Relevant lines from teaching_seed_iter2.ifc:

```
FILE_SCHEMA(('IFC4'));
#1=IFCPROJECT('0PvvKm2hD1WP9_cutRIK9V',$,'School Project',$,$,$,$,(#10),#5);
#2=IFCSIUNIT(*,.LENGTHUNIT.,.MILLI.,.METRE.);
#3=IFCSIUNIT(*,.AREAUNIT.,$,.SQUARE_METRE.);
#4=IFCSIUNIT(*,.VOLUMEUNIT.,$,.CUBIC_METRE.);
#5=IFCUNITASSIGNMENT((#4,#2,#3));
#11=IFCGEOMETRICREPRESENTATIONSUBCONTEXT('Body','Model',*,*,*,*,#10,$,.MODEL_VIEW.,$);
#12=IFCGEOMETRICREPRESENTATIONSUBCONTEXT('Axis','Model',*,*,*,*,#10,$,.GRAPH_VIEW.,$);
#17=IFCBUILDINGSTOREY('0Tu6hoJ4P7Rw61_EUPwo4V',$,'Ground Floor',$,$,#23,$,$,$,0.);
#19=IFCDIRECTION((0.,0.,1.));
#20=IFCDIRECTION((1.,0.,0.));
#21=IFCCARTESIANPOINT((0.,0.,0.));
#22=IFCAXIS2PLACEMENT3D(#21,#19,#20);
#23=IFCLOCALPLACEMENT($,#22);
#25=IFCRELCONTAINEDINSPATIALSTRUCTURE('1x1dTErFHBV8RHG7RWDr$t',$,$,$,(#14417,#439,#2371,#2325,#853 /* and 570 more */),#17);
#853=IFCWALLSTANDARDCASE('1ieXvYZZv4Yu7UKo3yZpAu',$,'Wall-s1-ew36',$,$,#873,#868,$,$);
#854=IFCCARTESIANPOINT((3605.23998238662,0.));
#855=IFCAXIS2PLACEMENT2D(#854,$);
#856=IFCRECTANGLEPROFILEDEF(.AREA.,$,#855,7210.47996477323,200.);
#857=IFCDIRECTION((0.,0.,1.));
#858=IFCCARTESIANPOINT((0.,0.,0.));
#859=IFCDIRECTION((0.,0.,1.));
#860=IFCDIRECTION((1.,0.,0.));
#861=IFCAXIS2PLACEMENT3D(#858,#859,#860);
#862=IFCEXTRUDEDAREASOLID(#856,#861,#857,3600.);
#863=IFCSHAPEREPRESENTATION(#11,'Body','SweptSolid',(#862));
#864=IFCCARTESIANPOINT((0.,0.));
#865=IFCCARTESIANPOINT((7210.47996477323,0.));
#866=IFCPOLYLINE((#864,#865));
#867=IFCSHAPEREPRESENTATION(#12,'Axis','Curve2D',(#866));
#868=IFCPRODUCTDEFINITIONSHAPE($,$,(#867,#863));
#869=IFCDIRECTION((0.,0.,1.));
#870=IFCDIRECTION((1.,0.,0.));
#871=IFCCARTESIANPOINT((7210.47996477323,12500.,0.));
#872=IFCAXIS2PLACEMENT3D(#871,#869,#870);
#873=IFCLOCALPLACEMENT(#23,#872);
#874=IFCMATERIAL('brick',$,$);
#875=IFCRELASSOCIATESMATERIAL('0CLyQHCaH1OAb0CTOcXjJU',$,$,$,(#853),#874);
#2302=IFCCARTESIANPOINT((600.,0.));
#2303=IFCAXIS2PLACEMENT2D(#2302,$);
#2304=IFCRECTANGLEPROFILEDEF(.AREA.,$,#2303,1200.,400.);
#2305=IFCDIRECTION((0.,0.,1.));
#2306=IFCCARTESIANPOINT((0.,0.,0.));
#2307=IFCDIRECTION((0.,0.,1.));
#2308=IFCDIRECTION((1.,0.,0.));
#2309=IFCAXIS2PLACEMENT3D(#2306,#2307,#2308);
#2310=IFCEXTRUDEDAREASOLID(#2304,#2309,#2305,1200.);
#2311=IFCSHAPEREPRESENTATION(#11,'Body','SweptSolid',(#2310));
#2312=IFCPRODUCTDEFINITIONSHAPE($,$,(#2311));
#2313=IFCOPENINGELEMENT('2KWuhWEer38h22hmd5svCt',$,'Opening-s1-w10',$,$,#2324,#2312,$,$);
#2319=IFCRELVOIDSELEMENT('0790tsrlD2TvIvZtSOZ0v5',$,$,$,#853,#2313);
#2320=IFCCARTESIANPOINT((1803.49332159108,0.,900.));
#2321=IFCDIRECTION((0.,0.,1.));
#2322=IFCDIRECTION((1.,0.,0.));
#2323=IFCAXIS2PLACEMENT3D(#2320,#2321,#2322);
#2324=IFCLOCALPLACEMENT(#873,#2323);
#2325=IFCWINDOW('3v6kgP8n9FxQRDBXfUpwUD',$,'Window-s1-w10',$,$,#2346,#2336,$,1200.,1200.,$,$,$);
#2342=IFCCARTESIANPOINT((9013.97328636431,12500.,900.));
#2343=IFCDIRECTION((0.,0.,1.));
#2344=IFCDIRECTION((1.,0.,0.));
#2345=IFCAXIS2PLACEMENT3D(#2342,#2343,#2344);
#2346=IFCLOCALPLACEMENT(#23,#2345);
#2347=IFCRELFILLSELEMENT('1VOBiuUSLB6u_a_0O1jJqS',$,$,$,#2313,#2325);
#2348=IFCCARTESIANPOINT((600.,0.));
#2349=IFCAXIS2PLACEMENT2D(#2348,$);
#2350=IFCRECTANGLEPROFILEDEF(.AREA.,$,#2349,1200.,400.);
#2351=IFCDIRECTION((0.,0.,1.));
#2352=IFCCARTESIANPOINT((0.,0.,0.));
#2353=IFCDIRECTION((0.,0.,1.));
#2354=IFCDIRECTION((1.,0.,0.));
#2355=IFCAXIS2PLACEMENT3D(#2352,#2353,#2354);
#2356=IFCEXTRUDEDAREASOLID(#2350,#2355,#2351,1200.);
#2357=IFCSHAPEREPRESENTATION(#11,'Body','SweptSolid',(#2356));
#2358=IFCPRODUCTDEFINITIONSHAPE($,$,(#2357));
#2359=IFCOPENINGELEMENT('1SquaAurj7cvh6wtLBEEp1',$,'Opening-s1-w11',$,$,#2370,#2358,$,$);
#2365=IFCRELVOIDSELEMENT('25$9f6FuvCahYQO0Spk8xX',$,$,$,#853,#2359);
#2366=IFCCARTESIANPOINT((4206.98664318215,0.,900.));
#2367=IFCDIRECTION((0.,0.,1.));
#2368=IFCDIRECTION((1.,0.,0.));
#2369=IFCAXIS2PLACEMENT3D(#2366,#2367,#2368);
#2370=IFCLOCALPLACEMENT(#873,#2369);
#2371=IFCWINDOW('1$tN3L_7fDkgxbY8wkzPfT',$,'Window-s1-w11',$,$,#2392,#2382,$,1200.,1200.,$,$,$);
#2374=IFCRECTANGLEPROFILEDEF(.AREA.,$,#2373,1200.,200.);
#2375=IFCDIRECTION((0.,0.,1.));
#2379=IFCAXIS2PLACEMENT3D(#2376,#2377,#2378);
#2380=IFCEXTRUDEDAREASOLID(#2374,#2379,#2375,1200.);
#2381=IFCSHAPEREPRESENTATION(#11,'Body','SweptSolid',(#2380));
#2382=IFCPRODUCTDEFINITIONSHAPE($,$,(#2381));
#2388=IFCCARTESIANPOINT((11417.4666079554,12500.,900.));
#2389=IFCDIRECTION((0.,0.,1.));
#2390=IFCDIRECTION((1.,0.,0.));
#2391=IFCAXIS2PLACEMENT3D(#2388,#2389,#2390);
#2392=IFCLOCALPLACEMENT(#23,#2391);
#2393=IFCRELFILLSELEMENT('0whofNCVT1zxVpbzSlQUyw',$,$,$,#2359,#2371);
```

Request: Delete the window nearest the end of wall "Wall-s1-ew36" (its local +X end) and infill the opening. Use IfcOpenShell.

```python
import ifcopenshell
import ifcopenshell.api.feature
import ifcopenshell.api.root
import ifcopenshell.geom
import ifcopenshell.util.shape

model = ifcopenshell.open("teaching_seed_iter2.ifc")
settings = ifcopenshell.geom.settings()


def volume(element):
    """Net volume in cubic metres, openings subtracted."""
    shape = ifcopenshell.geom.create_shape(settings, element)
    return ifcopenshell.util.shape.get_volume(shape.geometry)


window = model.by_guid("1$tN3L_7fDkgxbY8wkzPfT")
opening = window.FillsVoids[0].RelatingOpeningElement
wall = opening.VoidsElements[0].RelatingBuildingElement
before = volume(wall)

ifcopenshell.api.root.remove_product(model, product=window)
ifcopenshell.api.feature.remove_feature(model, feature=opening)

after = volume(wall)

print(f"wall volume {before:.3f} -> {after:.3f} m3")

model.write("teaching_seed_iter2_v2.ifc")
```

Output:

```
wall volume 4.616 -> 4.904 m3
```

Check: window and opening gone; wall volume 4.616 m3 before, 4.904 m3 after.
